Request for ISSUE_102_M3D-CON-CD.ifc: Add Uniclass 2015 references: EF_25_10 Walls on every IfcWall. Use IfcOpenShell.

First a look at what the model holds.

```python
import ifcopenshell

model = ifcopenshell.open("ISSUE_102_M3D-CON-CD.ifc")
print(model.schema)
print("classifications:", [c.Name for c in model.by_type("IfcClassification")])
for ifc_class in ("IfcDoor", "IfcRoof", "IfcStair", "IfcWall", "IfcWindow"):
    print(ifc_class, len(model.by_type(ifc_class)))
```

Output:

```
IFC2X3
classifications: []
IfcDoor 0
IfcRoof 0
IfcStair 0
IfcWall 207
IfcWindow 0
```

```python
import ifcopenshell
import ifcopenshell.api.classification

model = ifcopenshell.open("ISSUE_102_M3D-CON-CD.ifc")

# IFC2X3 requires Source and Edition and has no link from the project to the system.
system = model.create_entity("IfcClassification", Source="NBS", Edition="2015", Name="Uniclass 2015")

codes = {
    "IfcWall": ("EF_25_10", "Walls"),
}
for ifc_class, (code, name) in codes.items():
    products = model.by_type(ifc_class)
    ifcopenshell.api.classification.add_reference(
        model, products=products, classification=system, identification=code, name=name
    )
    print(code, len(products))

model.write("ISSUE_102_M3D-CON-CD_updated.ifc")
```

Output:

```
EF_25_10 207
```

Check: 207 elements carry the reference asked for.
